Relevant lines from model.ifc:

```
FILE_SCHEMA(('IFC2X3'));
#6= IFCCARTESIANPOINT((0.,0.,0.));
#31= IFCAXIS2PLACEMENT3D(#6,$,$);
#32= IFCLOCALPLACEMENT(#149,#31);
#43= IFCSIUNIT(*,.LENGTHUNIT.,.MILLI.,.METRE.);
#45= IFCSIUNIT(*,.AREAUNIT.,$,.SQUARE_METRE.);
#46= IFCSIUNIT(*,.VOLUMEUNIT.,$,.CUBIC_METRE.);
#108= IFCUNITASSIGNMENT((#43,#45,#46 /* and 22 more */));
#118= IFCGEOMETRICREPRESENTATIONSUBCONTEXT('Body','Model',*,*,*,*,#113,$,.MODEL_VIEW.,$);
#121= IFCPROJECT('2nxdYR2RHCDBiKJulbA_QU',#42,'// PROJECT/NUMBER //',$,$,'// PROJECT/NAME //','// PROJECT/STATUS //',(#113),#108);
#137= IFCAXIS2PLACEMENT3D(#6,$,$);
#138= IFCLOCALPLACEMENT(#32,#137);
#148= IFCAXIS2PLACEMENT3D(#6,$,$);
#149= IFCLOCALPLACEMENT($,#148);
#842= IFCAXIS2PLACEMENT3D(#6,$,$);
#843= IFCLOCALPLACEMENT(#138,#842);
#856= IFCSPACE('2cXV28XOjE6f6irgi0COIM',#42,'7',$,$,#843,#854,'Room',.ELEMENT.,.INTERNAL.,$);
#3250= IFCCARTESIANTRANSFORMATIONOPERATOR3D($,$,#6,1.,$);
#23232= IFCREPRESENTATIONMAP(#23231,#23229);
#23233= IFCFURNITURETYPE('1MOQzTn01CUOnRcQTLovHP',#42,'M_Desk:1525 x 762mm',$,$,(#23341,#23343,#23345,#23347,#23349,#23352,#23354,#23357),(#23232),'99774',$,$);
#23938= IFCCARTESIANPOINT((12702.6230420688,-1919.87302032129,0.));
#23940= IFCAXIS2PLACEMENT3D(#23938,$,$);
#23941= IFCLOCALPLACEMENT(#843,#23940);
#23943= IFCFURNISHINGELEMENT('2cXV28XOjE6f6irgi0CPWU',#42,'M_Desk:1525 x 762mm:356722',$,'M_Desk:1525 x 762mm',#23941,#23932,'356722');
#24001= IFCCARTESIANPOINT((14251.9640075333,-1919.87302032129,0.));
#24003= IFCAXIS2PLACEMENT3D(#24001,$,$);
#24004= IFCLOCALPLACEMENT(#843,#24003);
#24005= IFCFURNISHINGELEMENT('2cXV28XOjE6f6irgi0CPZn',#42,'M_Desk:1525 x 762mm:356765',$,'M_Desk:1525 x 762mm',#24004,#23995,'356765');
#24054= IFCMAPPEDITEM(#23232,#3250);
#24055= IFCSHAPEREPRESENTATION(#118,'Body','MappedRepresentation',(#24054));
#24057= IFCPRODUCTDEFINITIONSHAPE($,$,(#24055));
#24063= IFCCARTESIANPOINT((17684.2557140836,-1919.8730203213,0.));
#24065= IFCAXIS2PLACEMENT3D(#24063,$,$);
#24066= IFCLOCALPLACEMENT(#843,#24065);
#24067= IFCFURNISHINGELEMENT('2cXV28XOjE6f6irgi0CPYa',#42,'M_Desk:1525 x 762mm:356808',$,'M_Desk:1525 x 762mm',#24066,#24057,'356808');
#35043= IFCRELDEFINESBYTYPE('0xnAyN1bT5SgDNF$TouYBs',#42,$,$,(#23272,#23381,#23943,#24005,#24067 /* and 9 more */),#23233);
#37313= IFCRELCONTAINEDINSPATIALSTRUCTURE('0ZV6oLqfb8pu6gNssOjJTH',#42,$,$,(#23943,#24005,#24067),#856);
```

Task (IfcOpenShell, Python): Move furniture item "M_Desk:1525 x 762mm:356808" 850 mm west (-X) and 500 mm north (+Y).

```python
import ifcopenshell
import ifcopenshell.api.geometry
import ifcopenshell.util.placement
import ifcopenshell.util.unit

model = ifcopenshell.open("model.ifc")
unit_scale = ifcopenshell.util.unit.calculate_unit_scale(model)

item = model.by_id(24067)
matrix = ifcopenshell.util.placement.get_local_placement(item.ObjectPlacement)
matrix[0, 3] -= 0.85 / unit_scale
matrix[1, 3] += 0.5 / unit_scale
ifcopenshell.api.geometry.edit_object_placement(model, product=item, matrix=matrix, is_si=False)

print(ifcopenshell.util.placement.get_local_placement(item.ObjectPlacement).round(3) + 0.0)

model.write("model_rev.ifc")
```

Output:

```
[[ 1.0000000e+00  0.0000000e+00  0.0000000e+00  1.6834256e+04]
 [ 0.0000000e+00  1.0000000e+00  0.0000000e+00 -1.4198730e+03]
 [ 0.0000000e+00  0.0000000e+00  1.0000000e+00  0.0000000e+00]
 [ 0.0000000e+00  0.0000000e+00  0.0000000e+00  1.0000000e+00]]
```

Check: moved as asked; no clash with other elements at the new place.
